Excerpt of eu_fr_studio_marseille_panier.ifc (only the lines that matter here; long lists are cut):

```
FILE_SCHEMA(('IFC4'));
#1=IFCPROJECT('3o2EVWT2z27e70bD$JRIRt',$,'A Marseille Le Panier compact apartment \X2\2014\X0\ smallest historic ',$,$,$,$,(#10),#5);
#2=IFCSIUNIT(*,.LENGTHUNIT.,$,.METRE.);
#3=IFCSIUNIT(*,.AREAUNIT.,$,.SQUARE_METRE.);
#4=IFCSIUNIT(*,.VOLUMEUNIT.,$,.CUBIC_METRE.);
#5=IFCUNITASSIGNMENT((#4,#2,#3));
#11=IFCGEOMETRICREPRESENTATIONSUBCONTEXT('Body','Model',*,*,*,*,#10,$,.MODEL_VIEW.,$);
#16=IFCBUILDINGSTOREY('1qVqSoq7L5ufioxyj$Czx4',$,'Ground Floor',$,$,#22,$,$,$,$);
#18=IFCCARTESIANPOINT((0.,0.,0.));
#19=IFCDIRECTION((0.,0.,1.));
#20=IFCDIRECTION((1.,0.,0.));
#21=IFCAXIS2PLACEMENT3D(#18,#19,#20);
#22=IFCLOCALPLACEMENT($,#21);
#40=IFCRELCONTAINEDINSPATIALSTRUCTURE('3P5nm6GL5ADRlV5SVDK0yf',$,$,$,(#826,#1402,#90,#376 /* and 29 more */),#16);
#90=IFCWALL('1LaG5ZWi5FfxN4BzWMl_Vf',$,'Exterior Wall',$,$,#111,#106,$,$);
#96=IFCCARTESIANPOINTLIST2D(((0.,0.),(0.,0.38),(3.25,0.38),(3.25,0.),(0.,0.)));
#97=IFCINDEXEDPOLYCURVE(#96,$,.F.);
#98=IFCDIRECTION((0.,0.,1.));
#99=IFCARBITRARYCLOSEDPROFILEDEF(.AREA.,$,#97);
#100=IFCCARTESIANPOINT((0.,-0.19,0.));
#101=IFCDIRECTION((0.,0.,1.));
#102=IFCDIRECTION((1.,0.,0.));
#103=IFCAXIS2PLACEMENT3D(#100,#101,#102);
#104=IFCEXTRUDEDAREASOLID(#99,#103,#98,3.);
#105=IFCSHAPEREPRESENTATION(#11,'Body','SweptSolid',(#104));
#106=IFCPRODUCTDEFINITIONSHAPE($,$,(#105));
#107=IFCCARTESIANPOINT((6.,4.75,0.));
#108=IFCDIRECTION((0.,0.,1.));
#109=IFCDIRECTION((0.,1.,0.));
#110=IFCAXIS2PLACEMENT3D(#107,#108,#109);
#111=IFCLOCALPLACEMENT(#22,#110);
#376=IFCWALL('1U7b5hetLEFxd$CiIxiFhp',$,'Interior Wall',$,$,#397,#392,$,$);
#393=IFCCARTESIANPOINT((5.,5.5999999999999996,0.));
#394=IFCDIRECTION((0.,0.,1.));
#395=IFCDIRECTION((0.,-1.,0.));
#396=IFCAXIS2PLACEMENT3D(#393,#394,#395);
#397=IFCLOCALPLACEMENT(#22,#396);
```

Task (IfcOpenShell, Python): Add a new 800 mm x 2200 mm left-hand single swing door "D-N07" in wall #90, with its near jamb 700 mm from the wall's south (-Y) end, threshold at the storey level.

```python
import numpy as np
import ifcopenshell
import ifcopenshell.api.feature
import ifcopenshell.api.geometry
import ifcopenshell.api.root
import ifcopenshell.api.spatial
import ifcopenshell.geom
import ifcopenshell.util.element
import ifcopenshell.util.placement
import ifcopenshell.util.representation
import ifcopenshell.util.shape
import ifcopenshell.util.unit

model = ifcopenshell.open("eu_fr_studio_marseille_panier.ifc")
unit_scale = ifcopenshell.util.unit.calculate_unit_scale(model)
settings = ifcopenshell.geom.settings()


def volume(element):
    """Net volume in cubic metres, openings subtracted."""
    shape = ifcopenshell.geom.create_shape(settings, element)
    return ifcopenshell.util.shape.get_volume(shape.geometry)


wall = model.by_guid("1LaG5ZWi5FfxN4BzWMl_Vf")
storey = ifcopenshell.util.element.get_container(wall, ifc_class="IfcBuildingStorey")
context = ifcopenshell.util.representation.get_context(model, "Model", "Body", "MODEL_VIEW")
before = volume(wall)

width, height, from_end, sill = 0.8, 2.2, 0.7, 0.0  # metres

# The wall runs along its own X axis, and the end named is its -X end.
wall_shape = ifcopenshell.geom.create_shape(settings, wall)
x, y, z = ifcopenshell.util.shape.get_vertices(wall_shape.geometry).T
start = x.min() + from_end
face, thickness = float(y.min()), float(y.max() - y.min())
wall_matrix = ifcopenshell.util.placement.get_local_placement(wall.ObjectPlacement)
level = ifcopenshell.util.placement.get_local_placement(storey.ObjectPlacement)[2, 3]


def in_wall(x, y):
    """Placement at x, y metres in the wall's axes, at sill height."""
    matrix = wall_matrix.copy()
    matrix[:, 3] = wall_matrix @ np.array([x / unit_scale, y / unit_scale, 0.0, 1.0])
    matrix[2, 3] = level + sill / unit_scale
    return matrix


# Opening: a box that overshoots both wall faces by 50 mm.
opening = ifcopenshell.api.root.create_entity(model, ifc_class="IfcOpeningElement", predefined_type="OPENING")
box = ifcopenshell.api.geometry.add_wall_representation(
    model, context=context, length=width, height=height, thickness=thickness + 0.1
)
ifcopenshell.api.geometry.assign_representation(model, product=opening, representation=box)
ifcopenshell.api.geometry.edit_object_placement(model, product=opening, matrix=in_wall(start, face - 0.05), is_si=False)
ifcopenshell.api.feature.add_feature(model, feature=opening, element=wall)

door = ifcopenshell.api.root.create_entity(model, ifc_class="IfcDoor", name="D-N07", predefined_type="DOOR")
door.OverallWidth, door.OverallHeight = width / unit_scale, height / unit_scale
door.OperationType = "SINGLE_SWING_LEFT"
body = ifcopenshell.api.geometry.add_door_representation(
    model,
    context=context,
    overall_width=door.OverallWidth,
    overall_height=door.OverallHeight,
    operation_type="SINGLE_SWING_LEFT",
    lining_properties={"LiningDepth": thickness / unit_scale, "ThresholdDepth": thickness / unit_scale},
)
ifcopenshell.api.geometry.assign_representation(model, product=door, representation=body)
ifcopenshell.api.spatial.assign_container(model, products=[door], relating_structure=storey)
ifcopenshell.api.feature.add_filling(model, opening=opening, element=door)

# The lining spans the wall, so the door starts at the wall face.
ifcopenshell.api.geometry.edit_object_placement(model, product=door, matrix=in_wall(start, face), is_si=False)

after = volume(wall)

print(f"wall volume {before:.3f} -> {after:.3f} m3")

model.write("eu_fr_studio_marseille_panier_v2.ifc")
```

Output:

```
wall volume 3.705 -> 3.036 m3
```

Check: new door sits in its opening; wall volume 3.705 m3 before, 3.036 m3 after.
